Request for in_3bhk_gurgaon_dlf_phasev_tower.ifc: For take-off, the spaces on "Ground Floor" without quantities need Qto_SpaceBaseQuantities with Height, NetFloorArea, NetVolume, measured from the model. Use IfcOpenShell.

First a look at what the model holds.

```python
import ifcopenshell
import ifcopenshell.util.element
import ifcopenshell.util.unit

model = ifcopenshell.open("in_3bhk_gurgaon_dlf_phasev_tower.ifc")
print(model.schema)
for unit_type in ("LENGTHUNIT", "AREAUNIT", "VOLUMEUNIT"):
    print(unit_type, ifcopenshell.util.unit.calculate_unit_scale(model, unit_type))
storey = next(s for s in model.by_type("IfcBuildingStorey") if s.Name == "Ground Floor")
spaces = [e for e in ifcopenshell.util.element.get_decomposition(storey) if e.is_a("IfcSpace")]
for e in sorted(spaces, key=lambda e: e.id()):
    print(e.id(), e.is_a(), e.Name, list(ifcopenshell.util.element.get_psets(e, qtos_only=True)), sep=" | ")
```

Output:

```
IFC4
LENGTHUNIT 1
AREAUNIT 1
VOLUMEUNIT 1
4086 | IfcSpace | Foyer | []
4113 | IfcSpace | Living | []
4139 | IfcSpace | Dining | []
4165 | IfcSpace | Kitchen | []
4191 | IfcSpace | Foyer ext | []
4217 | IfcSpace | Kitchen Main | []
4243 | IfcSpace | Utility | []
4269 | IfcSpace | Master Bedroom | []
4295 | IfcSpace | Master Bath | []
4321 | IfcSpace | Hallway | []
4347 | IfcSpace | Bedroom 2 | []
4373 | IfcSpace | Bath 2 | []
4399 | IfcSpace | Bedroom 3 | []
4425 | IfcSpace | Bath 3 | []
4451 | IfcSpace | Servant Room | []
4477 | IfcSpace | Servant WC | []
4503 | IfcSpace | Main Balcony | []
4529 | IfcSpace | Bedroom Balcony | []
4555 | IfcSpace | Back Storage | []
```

```python
import ifcopenshell
import ifcopenshell.api.pset
import ifcopenshell.geom
import ifcopenshell.util.element
import ifcopenshell.util.shape
import ifcopenshell.util.unit

model = ifcopenshell.open("in_3bhk_gurgaon_dlf_phasev_tower.ifc")
unit_scale = ifcopenshell.util.unit.calculate_unit_scale(model)
area_scale = ifcopenshell.util.unit.calculate_unit_scale(model, "AREAUNIT")
volume_scale = ifcopenshell.util.unit.calculate_unit_scale(model, "VOLUMEUNIT")
settings = ifcopenshell.geom.settings()

storey = next(s for s in model.by_type("IfcBuildingStorey") if s.Name == "Ground Floor")
spaces = [e for e in ifcopenshell.util.element.get_decomposition(storey) if e.is_a("IfcSpace")]

for e in sorted(spaces, key=lambda e: e.id()):
    if ifcopenshell.util.element.get_psets(e, qtos_only=True, should_inherit=False):
        continue
    # Geometry comes back in metres, in the element's own axes.
    shape = ifcopenshell.geom.create_shape(settings, e)
    values = {
        "Height": ifcopenshell.util.shape.get_z(shape.geometry) / unit_scale,
        "NetFloorArea": ifcopenshell.util.shape.get_footprint_area(shape.geometry) / area_scale,
        "NetVolume": ifcopenshell.util.shape.get_volume(shape.geometry) / volume_scale,
    }
    qto = ifcopenshell.api.pset.add_qto(model, product=e, name="Qto_SpaceBaseQuantities")
    ifcopenshell.api.pset.edit_qto(model, qto=qto, properties=values)
    print(e.id(), {k: round(v, 3) for k, v in values.items()})

model.write("in_3bhk_gurgaon_dlf_phasev_tower_updated.ifc")
```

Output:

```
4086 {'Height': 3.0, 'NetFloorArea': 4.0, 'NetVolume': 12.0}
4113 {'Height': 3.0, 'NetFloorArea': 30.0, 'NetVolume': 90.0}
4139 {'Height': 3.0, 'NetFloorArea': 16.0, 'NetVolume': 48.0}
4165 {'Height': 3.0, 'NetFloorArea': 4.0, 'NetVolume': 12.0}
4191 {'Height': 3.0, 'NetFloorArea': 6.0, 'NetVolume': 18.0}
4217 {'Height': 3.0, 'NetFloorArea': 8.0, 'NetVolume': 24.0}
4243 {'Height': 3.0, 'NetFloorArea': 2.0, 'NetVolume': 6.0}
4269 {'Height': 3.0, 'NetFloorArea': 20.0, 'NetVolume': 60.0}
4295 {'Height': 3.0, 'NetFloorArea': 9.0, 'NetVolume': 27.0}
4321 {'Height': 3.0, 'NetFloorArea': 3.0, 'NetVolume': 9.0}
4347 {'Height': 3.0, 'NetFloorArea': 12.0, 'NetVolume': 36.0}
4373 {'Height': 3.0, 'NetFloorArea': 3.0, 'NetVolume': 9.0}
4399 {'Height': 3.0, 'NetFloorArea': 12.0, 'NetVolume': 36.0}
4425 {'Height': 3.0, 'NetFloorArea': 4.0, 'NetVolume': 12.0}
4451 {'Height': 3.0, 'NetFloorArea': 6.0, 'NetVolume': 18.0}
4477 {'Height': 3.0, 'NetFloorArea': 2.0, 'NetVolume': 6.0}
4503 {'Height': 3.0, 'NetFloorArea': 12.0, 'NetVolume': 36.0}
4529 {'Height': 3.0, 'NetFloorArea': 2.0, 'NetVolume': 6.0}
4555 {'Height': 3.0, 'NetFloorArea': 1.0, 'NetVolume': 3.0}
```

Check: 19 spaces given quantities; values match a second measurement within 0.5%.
